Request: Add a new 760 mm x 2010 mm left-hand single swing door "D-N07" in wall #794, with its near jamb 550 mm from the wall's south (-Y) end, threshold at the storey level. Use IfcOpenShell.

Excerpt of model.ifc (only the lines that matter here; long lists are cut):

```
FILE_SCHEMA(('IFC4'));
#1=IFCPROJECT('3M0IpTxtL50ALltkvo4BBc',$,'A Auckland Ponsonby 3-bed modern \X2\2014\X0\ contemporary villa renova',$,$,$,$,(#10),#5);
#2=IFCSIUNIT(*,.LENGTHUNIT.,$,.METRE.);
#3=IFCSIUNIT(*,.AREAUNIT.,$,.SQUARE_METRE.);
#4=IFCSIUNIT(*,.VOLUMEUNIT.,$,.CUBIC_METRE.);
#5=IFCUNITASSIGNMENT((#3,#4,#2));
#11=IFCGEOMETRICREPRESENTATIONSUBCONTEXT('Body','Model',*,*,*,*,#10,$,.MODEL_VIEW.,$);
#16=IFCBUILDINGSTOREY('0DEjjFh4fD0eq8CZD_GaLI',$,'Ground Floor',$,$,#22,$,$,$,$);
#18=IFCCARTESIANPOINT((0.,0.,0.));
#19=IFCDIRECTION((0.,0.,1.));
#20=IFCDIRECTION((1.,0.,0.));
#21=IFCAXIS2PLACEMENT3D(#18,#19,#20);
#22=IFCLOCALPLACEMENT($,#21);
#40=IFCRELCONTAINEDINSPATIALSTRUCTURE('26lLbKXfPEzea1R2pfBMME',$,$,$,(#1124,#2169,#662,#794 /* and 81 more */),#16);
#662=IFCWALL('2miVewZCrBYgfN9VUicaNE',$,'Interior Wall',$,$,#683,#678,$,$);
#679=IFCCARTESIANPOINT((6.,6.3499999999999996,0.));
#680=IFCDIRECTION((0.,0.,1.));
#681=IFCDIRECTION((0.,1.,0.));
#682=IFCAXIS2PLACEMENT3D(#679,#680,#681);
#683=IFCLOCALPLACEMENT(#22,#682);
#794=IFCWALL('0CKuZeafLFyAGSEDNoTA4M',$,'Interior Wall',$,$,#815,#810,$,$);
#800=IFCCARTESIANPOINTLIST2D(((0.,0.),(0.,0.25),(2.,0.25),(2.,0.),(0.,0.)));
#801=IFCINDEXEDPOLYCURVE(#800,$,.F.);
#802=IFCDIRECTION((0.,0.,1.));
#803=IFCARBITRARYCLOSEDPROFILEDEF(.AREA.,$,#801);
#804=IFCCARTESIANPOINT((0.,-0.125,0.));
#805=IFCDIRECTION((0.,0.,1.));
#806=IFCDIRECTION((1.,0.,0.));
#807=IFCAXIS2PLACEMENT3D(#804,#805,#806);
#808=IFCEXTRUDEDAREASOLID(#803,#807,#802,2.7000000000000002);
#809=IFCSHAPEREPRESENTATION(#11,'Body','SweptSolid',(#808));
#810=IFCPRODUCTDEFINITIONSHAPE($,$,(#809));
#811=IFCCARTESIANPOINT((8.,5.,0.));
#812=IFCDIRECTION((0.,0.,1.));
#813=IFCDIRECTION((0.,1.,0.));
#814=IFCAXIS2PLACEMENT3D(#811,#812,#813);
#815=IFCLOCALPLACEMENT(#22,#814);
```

```python
import numpy as np
import ifcopenshell
import ifcopenshell.api.feature
import ifcopenshell.api.geometry
import ifcopenshell.api.root
import ifcopenshell.api.spatial
import ifcopenshell.geom
import ifcopenshell.util.element
import ifcopenshell.util.placement
import ifcopenshell.util.representation
import ifcopenshell.util.shape
import ifcopenshell.util.unit

model = ifcopenshell.open("model.ifc")
unit_scale = ifcopenshell.util.unit.calculate_unit_scale(model)
settings = ifcopenshell.geom.settings()


def volume(element):
    """Net volume in cubic metres, openings subtracted."""
    shape = ifcopenshell.geom.create_shape(settings, element)
    return ifcopenshell.util.shape.get_volume(shape.geometry)


wall = model.by_guid("0CKuZeafLFyAGSEDNoTA4M")
storey = ifcopenshell.util.element.get_container(wall, ifc_class="IfcBuildingStorey")
context = ifcopenshell.util.representation.get_context(model, "Model", "Body", "MODEL_VIEW")
before = volume(wall)

width, height, from_end, sill = 0.76, 2.01, 0.55, 0.0  # metres

# The wall runs along its own X axis, and the end named is its -X end.
wall_shape = ifcopenshell.geom.create_shape(settings, wall)
x, y, z = ifcopenshell.util.shape.get_vertices(wall_shape.geometry).T
start = x.min() + from_end
face, thickness = float(y.min()), float(y.max() - y.min())
wall_matrix = ifcopenshell.util.placement.get_local_placement(wall.ObjectPlacement)
level = ifcopenshell.util.placement.get_local_placement(storey.ObjectPlacement)[2, 3]


def in_wall(x, y):
    """Placement at x, y metres in the wall's axes, at sill height."""
    matrix = wall_matrix.copy()
    matrix[:, 3] = wall_matrix @ np.array([x / unit_scale, y / unit_scale, 0.0, 1.0])
    matrix[2, 3] = level + sill / unit_scale
    return matrix


# Opening: a box that overshoots both wall faces by 50 mm.
opening = ifcopenshell.api.root.create_entity(model, ifc_class="IfcOpeningElement", predefined_type="OPENING")
box = ifcopenshell.api.geometry.add_wall_representation(
    model, context=context, length=width, height=height, thickness=thickness + 0.1
)
ifcopenshell.api.geometry.assign_representation(model, product=opening, representation=box)
ifcopenshell.api.geometry.edit_object_placement(model, product=opening, matrix=in_wall(start, face - 0.05), is_si=False)
ifcopenshell.api.feature.add_feature(model, feature=opening, element=wall)

door = ifcopenshell.api.root.create_entity(model, ifc_class="IfcDoor", name="D-N07", predefined_type="DOOR")
door.OverallWidth, door.OverallHeight = width / unit_scale, height / unit_scale
door.OperationType = "SINGLE_SWING_LEFT"
body = ifcopenshell.api.geometry.add_door_representation(
    model,
    context=context,
    overall_width=door.OverallWidth,
    overall_height=door.OverallHeight,
    operation_type="SINGLE_SWING_LEFT",
    lining_properties={"LiningDepth": thickness / unit_scale, "ThresholdDepth": thickness / unit_scale},
)
ifcopenshell.api.geometry.assign_representation(model, product=door, representation=body)
ifcopenshell.api.spatial.assign_container(model, products=[door], relating_structure=storey)
ifcopenshell.api.feature.add_filling(model, opening=opening, element=door)

# The lining spans the wall, so the door starts at the wall face.
ifcopenshell.api.geometry.edit_object_placement(model, product=door, matrix=in_wall(start, face), is_si=False)

after = volume(wall)

print(f"wall volume {before:.3f} -> {after:.3f} m3")

model.write("model_rev.ifc")
```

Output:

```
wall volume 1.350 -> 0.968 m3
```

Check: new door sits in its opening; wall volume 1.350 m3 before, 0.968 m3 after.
